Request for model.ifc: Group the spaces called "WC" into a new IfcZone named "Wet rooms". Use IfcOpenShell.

First a look at what the model holds.

```python
import ifcopenshell

model = ifcopenshell.open("model.ifc")
print(model.schema)
seen = {}
for space in model.by_type("IfcSpace"):
    seen[space.LongName] = seen.get(space.LongName, 0) + 1
for name, count in sorted(seen.items(), key=str):
    print(count, "x", name)
print("zones:", [z.Name for z in model.by_type("IfcZone")][:20])
```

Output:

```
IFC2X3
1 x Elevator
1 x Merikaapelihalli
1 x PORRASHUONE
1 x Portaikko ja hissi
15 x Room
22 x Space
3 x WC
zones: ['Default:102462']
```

```python
import ifcopenshell
import ifcopenshell.api.group
import ifcopenshell.api.root

model = ifcopenshell.open("model.ifc")

names = {"WC"}
spaces = [s for s in model.by_type("IfcSpace") if s.LongName in names]

zone = ifcopenshell.api.root.create_entity(model, ifc_class="IfcZone", name="Wet rooms")
ifcopenshell.api.group.assign_group(model, products=spaces, group=zone)
print(len(spaces), "spaces in", zone.Name)

model.write("model_edited.ifc")
```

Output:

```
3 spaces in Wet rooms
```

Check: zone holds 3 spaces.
